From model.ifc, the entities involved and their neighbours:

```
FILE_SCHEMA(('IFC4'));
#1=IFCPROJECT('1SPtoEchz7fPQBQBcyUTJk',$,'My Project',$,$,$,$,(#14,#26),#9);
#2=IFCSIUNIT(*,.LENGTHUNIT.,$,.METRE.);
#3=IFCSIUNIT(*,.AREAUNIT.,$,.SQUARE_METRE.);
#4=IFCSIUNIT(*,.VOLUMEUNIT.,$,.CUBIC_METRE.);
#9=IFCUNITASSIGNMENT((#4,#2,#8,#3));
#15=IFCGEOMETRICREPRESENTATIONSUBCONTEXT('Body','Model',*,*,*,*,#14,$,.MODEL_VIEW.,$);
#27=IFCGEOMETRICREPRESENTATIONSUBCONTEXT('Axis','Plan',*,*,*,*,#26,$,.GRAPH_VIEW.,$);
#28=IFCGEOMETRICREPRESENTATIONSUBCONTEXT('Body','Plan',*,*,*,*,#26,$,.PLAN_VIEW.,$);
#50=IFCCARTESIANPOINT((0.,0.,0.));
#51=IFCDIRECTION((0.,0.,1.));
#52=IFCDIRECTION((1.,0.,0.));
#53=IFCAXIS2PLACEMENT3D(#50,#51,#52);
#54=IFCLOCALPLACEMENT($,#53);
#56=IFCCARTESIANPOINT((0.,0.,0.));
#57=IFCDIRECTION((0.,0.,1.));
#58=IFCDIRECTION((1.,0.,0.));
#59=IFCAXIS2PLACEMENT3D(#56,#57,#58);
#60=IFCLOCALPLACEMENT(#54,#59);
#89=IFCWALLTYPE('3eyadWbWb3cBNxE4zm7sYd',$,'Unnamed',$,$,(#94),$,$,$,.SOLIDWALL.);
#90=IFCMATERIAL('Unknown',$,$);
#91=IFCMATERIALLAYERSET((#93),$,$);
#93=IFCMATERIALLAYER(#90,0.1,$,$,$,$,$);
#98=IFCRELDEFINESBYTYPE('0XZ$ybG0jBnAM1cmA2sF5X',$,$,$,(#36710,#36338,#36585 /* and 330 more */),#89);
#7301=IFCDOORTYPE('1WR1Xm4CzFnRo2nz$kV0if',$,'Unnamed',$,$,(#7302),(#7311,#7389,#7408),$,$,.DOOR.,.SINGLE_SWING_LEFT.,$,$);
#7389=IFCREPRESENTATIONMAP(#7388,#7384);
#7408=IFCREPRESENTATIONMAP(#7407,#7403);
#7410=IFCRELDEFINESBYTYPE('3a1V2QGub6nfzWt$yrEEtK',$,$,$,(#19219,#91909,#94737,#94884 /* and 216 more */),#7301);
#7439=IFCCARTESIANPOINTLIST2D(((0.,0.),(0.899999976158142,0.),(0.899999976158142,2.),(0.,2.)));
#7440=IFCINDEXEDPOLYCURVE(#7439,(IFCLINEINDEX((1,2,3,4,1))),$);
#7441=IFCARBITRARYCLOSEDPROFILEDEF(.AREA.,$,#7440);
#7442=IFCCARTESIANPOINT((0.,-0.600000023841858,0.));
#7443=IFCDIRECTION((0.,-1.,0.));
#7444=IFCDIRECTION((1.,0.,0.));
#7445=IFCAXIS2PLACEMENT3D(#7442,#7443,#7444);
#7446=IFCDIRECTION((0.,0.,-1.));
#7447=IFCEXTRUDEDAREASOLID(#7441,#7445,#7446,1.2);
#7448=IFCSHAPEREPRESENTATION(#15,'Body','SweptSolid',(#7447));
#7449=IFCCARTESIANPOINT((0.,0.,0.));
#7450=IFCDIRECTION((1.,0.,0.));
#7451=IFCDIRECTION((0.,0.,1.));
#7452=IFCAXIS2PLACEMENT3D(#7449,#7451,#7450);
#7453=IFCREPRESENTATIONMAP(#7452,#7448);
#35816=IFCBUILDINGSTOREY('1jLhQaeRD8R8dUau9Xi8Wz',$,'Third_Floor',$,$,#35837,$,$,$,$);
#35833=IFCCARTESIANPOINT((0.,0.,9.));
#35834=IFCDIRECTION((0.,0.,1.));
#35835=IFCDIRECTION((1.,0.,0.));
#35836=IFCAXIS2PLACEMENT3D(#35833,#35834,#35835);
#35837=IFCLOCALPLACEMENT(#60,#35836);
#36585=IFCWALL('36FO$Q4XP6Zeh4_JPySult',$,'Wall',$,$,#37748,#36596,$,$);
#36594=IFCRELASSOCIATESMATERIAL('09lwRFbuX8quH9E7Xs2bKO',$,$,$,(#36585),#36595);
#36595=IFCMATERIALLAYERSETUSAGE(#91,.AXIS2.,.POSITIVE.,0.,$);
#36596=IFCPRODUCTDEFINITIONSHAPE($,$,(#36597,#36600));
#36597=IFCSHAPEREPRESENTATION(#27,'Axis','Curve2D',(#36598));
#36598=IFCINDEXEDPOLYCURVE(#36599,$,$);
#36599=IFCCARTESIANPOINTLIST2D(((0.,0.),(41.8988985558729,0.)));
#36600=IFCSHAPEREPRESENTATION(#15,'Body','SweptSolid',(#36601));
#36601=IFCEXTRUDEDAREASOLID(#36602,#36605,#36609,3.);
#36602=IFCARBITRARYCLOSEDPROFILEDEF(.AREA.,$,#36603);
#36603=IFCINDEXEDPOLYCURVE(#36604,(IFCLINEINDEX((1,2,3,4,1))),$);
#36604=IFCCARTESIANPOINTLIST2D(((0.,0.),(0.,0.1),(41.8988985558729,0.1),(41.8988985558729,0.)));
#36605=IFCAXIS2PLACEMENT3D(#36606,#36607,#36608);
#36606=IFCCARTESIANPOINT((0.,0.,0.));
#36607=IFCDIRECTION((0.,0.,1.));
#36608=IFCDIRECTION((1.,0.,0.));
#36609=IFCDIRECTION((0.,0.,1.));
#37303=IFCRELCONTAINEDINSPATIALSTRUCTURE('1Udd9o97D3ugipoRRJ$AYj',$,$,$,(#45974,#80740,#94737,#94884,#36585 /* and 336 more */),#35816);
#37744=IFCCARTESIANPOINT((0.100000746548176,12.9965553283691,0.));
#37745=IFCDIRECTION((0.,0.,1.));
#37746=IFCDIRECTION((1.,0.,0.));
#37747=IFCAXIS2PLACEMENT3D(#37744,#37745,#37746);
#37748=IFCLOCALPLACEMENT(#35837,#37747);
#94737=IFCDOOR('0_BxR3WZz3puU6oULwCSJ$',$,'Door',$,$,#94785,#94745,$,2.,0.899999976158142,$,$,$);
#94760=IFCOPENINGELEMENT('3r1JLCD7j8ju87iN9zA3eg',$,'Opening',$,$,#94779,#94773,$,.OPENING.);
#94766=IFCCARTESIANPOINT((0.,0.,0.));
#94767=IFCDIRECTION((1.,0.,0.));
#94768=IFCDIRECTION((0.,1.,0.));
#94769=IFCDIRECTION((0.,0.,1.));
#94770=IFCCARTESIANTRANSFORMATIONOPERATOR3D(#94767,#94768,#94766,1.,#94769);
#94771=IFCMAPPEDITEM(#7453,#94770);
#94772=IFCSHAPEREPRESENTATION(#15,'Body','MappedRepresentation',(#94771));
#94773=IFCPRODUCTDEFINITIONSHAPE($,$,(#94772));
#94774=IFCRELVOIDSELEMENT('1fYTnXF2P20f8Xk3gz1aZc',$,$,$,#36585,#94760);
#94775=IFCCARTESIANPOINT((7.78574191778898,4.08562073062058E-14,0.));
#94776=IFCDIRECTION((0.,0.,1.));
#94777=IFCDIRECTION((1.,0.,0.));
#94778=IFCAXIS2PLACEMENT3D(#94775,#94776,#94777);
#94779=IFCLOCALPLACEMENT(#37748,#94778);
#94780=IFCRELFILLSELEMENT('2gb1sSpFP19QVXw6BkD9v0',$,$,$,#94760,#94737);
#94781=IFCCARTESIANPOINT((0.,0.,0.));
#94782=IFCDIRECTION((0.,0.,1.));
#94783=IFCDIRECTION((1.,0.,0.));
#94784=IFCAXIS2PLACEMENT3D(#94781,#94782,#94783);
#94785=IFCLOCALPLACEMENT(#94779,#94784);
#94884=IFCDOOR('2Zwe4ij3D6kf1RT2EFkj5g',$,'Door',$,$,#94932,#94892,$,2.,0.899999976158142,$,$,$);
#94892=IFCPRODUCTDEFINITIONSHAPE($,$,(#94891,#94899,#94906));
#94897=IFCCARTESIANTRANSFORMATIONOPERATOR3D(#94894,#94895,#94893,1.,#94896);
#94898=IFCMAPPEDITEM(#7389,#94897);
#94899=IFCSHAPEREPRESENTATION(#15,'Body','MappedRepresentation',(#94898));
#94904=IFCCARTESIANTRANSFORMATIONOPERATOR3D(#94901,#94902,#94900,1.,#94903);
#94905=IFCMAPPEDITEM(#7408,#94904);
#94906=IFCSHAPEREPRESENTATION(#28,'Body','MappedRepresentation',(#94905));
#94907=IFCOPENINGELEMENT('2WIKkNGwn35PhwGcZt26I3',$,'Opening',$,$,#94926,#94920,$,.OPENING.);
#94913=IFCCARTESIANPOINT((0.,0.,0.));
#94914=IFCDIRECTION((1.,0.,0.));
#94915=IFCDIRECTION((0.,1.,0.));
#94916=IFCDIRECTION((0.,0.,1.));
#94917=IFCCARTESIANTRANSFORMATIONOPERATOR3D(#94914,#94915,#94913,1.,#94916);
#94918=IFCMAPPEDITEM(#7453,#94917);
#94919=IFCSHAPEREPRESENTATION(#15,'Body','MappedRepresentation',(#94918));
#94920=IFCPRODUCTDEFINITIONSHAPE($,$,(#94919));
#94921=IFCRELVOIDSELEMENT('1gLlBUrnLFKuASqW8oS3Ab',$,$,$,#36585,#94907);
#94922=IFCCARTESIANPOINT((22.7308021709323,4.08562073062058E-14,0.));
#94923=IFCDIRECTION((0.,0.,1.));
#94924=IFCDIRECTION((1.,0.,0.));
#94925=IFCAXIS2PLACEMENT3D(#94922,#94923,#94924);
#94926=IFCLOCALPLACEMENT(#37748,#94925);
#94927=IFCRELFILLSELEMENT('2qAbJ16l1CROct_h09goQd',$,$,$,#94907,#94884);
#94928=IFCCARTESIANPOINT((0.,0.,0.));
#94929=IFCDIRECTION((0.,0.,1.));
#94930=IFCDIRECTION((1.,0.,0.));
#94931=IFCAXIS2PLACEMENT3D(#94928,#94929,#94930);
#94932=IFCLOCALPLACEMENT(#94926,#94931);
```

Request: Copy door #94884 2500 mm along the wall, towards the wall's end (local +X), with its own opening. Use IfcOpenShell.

```python
import ifcopenshell
import ifcopenshell.api.feature
import ifcopenshell.api.geometry
import ifcopenshell.api.root
import ifcopenshell.geom
import ifcopenshell.util.element
import ifcopenshell.util.placement
import ifcopenshell.util.shape

model = ifcopenshell.open("model.ifc")
settings = ifcopenshell.geom.settings()


def volume(element):
    """Net volume in cubic metres, openings subtracted."""
    shape = ifcopenshell.geom.create_shape(settings, element)
    return ifcopenshell.util.shape.get_volume(shape.geometry)


door = model.by_id(94884)
opening = door.FillsVoids[0].RelatingOpeningElement
wall = opening.VoidsElements[0].RelatingBuildingElement
before = volume(wall)
shift = ifcopenshell.util.placement.get_local_placement(wall.ObjectPlacement)[:3, 0] * 2.5

# copy_class copies the void relationship, type, container and properties, but no geometry.
new_opening = ifcopenshell.api.root.copy_class(model, product=opening)
new_opening.Representation = ifcopenshell.util.element.copy_deep(
    model, opening.Representation, exclude=["IfcGeometricRepresentationContext", "IfcRepresentationMap"]
)
new_door = ifcopenshell.api.root.copy_class(model, product=door)
new_door.Representation = ifcopenshell.util.element.copy_deep(
    model, door.Representation, exclude=["IfcGeometricRepresentationContext", "IfcRepresentationMap"]
)
ifcopenshell.api.feature.add_filling(model, opening=new_opening, element=new_door)

for old, new in ((opening, new_opening), (door, new_door)):
    matrix = ifcopenshell.util.placement.get_local_placement(old.ObjectPlacement)
    matrix[:3, 3] += shift
    ifcopenshell.api.geometry.edit_object_placement(model, product=new, matrix=matrix, is_si=False)

after = volume(wall)

print(f"wall volume {before:.3f} -> {after:.3f} m3")

model.write("model-out.ifc")
```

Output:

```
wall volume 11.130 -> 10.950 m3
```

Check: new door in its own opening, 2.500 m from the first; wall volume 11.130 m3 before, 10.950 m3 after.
